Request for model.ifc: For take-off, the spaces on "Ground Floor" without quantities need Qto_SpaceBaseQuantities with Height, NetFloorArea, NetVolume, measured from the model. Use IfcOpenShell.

First a look at what the model holds.

```python
import ifcopenshell
import ifcopenshell.util.element
import ifcopenshell.util.unit

model = ifcopenshell.open("model.ifc")
print(model.schema)
for unit_type in ("LENGTHUNIT", "AREAUNIT", "VOLUMEUNIT"):
    print(unit_type, ifcopenshell.util.unit.calculate_unit_scale(model, unit_type))
storey = next(s for s in model.by_type("IfcBuildingStorey") if s.Name == "Ground Floor")
spaces = [e for e in ifcopenshell.util.element.get_decomposition(storey) if e.is_a("IfcSpace")]
for e in sorted(spaces, key=lambda e: e.id()):
    print(e.id(), e.is_a(), e.Name, list(ifcopenshell.util.element.get_psets(e, qtos_only=True)), sep=" | ")
```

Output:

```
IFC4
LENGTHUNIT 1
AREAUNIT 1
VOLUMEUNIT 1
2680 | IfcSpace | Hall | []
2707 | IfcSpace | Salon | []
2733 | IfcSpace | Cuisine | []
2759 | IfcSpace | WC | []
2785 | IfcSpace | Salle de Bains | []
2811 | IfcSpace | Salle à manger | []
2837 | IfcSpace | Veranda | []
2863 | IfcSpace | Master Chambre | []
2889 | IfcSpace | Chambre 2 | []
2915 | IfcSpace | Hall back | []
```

```python
import ifcopenshell
import ifcopenshell.api.pset
import ifcopenshell.geom
import ifcopenshell.util.element
import ifcopenshell.util.shape
import ifcopenshell.util.unit

model = ifcopenshell.open("model.ifc")
unit_scale = ifcopenshell.util.unit.calculate_unit_scale(model)
area_scale = ifcopenshell.util.unit.calculate_unit_scale(model, "AREAUNIT")
volume_scale = ifcopenshell.util.unit.calculate_unit_scale(model, "VOLUMEUNIT")
settings = ifcopenshell.geom.settings()

storey = next(s for s in model.by_type("IfcBuildingStorey") if s.Name == "Ground Floor")
spaces = [e for e in ifcopenshell.util.element.get_decomposition(storey) if e.is_a("IfcSpace")]

for e in sorted(spaces, key=lambda e: e.id()):
    if ifcopenshell.util.element.get_psets(e, qtos_only=True, should_inherit=False):
        continue
    # Geometry comes back in metres, in the element's own axes.
    shape = ifcopenshell.geom.create_shape(settings, e)
    values = {
        "Height": ifcopenshell.util.shape.get_z(shape.geometry) / unit_scale,
        "NetFloorArea": ifcopenshell.util.shape.get_footprint_area(shape.geometry) / area_scale,
        "NetVolume": ifcopenshell.util.shape.get_volume(shape.geometry) / volume_scale,
    }
    qto = ifcopenshell.api.pset.add_qto(model, product=e, name="Qto_SpaceBaseQuantities")
    ifcopenshell.api.pset.edit_qto(model, qto=qto, properties=values)
    print(e.id(), {k: round(v, 3) for k, v in values.items()})

model.write("model_rev.ifc")
```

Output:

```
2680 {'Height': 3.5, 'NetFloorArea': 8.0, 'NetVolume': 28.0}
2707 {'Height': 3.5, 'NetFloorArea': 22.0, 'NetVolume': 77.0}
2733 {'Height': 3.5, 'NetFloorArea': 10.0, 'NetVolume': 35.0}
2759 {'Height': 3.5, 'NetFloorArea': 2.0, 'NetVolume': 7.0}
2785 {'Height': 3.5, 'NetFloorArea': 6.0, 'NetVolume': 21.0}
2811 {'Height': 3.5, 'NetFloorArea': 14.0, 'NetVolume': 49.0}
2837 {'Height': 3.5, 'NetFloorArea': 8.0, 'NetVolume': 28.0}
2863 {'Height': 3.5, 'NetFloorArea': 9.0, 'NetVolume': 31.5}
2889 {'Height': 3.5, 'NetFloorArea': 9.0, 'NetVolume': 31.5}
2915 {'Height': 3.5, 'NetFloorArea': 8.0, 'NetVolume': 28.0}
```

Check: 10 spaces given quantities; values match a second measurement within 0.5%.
